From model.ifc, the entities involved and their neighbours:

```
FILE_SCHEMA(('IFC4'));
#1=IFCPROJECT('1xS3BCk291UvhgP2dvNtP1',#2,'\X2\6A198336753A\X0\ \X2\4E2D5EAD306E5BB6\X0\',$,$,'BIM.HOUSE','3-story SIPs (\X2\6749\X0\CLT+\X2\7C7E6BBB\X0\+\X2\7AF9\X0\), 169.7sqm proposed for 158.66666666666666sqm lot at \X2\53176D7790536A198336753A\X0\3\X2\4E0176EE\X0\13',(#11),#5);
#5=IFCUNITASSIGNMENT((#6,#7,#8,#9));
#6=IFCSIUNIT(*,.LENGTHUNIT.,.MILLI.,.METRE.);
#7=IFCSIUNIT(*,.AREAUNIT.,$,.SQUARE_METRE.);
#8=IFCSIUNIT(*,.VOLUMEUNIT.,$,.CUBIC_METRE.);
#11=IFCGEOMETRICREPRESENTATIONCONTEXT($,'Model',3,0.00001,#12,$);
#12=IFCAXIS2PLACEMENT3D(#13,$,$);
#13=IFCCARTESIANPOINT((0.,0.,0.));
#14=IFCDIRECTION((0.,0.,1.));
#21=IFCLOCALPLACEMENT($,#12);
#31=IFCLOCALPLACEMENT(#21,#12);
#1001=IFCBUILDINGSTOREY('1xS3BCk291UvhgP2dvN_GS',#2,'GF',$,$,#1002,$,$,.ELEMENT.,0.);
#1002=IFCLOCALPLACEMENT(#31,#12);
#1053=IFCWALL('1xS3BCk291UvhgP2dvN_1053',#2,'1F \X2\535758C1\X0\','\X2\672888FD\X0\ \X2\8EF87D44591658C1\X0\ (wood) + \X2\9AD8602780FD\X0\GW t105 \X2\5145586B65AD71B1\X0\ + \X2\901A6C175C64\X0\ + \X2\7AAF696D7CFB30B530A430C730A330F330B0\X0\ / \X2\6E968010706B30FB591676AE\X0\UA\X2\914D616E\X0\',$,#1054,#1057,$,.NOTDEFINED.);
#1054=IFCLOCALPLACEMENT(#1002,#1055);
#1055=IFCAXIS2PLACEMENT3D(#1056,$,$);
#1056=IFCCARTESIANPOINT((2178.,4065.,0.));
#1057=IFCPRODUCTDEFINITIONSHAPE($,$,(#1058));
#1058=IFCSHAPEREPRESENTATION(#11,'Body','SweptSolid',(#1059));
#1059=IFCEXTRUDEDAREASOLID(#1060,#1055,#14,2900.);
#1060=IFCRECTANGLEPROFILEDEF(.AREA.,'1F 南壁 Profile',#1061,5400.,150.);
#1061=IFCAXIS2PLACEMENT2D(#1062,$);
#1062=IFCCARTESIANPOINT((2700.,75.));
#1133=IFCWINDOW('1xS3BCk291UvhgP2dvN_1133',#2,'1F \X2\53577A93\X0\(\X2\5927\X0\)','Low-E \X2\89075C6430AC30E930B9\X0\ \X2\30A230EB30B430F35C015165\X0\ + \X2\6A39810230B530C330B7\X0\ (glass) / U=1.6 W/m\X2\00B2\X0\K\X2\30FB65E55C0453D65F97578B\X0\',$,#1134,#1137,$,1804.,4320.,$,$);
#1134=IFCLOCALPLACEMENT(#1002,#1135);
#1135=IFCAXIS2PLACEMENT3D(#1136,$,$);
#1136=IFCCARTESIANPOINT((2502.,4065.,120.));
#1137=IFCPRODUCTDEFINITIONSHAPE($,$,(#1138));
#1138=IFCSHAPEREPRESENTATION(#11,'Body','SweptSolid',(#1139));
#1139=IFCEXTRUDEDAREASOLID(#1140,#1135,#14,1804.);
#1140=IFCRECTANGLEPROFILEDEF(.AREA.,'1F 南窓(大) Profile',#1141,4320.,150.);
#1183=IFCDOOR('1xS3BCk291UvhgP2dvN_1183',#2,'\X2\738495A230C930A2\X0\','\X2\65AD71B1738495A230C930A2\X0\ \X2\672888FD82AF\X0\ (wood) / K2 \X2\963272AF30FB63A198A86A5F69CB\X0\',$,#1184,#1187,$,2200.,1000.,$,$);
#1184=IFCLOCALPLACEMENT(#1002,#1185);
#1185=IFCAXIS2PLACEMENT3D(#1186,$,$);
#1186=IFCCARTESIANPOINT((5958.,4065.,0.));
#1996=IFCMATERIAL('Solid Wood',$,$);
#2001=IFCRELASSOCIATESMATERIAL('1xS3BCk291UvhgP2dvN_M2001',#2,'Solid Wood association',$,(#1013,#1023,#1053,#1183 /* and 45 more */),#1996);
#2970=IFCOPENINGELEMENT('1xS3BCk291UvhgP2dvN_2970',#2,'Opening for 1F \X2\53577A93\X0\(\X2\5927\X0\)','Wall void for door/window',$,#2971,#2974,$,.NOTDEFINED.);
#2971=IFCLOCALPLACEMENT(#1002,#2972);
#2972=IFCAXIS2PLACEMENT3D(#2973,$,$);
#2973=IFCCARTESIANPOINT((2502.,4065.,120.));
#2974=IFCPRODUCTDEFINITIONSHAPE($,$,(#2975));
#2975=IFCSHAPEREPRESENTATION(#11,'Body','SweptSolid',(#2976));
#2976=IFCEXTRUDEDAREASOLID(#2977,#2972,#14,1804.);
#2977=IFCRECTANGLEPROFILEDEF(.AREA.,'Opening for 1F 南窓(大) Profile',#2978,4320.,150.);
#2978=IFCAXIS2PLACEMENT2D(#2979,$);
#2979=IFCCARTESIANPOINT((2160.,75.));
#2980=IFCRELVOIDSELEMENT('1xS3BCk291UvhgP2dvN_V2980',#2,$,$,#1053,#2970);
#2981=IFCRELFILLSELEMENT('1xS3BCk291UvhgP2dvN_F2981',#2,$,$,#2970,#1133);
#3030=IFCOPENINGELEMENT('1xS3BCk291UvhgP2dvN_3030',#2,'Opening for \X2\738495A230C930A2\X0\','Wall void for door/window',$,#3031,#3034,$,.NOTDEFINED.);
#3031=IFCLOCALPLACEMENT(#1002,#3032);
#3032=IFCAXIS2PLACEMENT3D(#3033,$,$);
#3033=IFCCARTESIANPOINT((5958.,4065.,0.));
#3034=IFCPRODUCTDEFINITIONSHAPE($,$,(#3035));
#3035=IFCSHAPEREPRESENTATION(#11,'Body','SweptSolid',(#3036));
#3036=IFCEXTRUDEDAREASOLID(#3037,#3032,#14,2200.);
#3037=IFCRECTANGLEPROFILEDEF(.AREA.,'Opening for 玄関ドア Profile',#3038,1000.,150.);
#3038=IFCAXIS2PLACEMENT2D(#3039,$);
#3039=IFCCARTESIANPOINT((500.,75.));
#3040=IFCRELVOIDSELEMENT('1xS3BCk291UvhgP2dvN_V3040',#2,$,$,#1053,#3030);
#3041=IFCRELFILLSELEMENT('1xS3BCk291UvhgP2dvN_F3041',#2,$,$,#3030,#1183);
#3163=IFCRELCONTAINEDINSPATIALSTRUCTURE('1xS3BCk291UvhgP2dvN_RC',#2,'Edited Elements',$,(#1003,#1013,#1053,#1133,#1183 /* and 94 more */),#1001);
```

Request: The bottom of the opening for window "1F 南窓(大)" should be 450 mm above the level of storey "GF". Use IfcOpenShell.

```python
import numpy as np
import ifcopenshell
import ifcopenshell.api.geometry
import ifcopenshell.geom
import ifcopenshell.util.element
import ifcopenshell.util.placement
import ifcopenshell.util.shape
import ifcopenshell.util.unit

model = ifcopenshell.open("model.ifc")
unit_scale = ifcopenshell.util.unit.calculate_unit_scale(model)

window = model.by_guid("1xS3BCk291UvhgP2dvN_1133")
opening = window.FillsVoids[0].RelatingOpeningElement
storey = ifcopenshell.util.element.get_container(window, ifc_class="IfcBuildingStorey")
level = ifcopenshell.util.placement.get_local_placement(storey.ObjectPlacement)[2, 3]

# The opening's origin need not be at the sill, so measure its lowest point.
shape = ifcopenshell.geom.create_shape(ifcopenshell.geom.settings(), opening)
bottom = ifcopenshell.util.shape.get_shape_bottom_elevation(shape, shape.geometry) / unit_scale
dz = level + 0.45 / unit_scale - bottom

shift = np.array([0.0, 0.0, dz])
# The window is not placed relative to its opening, so move both.
for product in (opening, window):
    matrix = ifcopenshell.util.placement.get_local_placement(product.ObjectPlacement)
    matrix[:3, 3] += shift
    ifcopenshell.api.geometry.edit_object_placement(model, product=product, matrix=matrix, is_si=False)

print(f"moved by {dz * unit_scale:+.3f} m")

model.write("model_rev.ifc")
```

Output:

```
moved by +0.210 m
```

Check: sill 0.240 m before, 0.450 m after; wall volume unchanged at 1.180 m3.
